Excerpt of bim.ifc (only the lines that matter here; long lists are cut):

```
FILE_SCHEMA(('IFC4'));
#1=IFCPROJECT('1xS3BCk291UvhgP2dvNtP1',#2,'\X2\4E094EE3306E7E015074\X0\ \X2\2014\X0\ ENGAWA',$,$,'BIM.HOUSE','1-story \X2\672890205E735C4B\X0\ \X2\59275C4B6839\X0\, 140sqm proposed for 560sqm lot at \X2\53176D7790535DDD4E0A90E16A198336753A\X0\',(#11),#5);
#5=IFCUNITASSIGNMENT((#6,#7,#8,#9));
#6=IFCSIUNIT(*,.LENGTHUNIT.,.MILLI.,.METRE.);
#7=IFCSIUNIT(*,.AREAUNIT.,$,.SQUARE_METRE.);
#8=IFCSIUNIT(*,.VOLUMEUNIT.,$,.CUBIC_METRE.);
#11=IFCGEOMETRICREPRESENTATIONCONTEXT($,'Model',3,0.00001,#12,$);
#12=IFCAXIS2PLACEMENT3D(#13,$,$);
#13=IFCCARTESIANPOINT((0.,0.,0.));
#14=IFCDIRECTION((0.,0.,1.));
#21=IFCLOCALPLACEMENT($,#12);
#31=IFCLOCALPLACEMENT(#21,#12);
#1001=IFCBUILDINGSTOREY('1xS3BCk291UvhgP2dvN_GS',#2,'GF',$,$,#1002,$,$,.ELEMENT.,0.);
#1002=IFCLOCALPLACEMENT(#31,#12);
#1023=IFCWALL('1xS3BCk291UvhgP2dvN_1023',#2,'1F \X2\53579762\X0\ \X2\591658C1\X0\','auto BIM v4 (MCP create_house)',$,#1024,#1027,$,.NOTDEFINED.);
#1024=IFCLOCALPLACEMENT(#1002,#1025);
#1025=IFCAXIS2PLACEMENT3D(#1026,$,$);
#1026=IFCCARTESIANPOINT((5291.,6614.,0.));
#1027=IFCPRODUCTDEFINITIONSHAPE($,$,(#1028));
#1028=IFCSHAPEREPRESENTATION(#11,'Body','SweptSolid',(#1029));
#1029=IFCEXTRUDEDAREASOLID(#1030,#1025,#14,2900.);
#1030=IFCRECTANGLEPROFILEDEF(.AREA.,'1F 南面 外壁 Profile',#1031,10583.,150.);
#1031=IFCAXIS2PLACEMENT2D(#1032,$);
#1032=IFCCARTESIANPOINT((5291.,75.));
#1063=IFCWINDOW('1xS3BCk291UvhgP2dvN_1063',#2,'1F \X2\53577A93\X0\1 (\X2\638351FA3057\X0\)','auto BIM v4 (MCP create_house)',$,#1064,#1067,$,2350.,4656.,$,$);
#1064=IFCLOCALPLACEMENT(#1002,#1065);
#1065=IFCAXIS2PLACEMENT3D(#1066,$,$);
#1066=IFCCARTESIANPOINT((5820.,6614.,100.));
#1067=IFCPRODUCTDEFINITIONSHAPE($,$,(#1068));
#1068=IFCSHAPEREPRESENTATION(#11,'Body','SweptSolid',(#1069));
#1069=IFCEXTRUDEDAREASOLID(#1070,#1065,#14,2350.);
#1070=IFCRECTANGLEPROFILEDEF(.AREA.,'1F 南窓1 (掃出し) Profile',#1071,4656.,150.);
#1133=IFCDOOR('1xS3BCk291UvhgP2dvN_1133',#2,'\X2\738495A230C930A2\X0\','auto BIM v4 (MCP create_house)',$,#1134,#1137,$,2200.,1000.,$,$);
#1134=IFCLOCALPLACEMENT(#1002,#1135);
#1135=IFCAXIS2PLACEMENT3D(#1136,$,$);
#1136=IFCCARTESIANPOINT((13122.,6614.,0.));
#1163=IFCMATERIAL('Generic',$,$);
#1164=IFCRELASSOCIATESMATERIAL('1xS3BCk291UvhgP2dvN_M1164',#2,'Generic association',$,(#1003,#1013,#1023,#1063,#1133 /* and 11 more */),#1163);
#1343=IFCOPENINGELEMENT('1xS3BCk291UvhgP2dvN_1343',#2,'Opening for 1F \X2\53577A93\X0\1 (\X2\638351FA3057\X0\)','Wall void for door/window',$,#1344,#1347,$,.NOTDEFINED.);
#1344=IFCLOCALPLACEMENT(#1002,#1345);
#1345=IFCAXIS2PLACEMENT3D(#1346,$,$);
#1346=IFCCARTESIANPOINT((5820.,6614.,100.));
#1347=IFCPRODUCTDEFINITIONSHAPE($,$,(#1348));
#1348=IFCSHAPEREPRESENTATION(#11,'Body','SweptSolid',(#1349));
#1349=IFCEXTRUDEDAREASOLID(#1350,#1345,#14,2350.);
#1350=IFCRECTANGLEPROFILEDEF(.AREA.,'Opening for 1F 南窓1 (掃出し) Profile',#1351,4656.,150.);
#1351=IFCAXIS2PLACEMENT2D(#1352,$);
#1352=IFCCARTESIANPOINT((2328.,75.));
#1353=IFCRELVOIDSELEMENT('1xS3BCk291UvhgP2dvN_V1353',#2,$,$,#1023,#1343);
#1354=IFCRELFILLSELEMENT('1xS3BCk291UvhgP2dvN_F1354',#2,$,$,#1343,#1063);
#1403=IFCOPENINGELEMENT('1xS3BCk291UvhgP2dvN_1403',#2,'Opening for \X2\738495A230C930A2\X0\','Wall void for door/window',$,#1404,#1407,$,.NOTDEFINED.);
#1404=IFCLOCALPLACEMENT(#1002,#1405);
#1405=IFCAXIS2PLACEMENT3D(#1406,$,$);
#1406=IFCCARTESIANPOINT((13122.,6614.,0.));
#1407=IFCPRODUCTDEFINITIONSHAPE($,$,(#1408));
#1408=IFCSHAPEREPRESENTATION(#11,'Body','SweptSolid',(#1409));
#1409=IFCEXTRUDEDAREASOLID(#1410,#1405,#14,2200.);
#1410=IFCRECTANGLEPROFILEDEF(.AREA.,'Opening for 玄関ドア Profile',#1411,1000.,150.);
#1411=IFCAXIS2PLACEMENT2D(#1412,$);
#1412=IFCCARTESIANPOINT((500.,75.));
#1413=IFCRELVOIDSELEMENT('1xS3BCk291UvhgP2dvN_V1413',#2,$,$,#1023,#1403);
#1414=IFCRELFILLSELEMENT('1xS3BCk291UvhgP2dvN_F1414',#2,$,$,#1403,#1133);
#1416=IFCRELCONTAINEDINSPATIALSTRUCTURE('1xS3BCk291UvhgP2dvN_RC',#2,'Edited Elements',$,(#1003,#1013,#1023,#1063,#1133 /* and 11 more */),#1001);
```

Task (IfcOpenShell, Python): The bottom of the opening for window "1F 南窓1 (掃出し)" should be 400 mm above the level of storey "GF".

```python
import numpy as np
import ifcopenshell
import ifcopenshell.api.geometry
import ifcopenshell.geom
import ifcopenshell.util.element
import ifcopenshell.util.placement
import ifcopenshell.util.shape
import ifcopenshell.util.unit

model = ifcopenshell.open("bim.ifc")
unit_scale = ifcopenshell.util.unit.calculate_unit_scale(model)

window = model.by_guid("1xS3BCk291UvhgP2dvN_1063")
opening = window.FillsVoids[0].RelatingOpeningElement
storey = ifcopenshell.util.element.get_container(window, ifc_class="IfcBuildingStorey")
level = ifcopenshell.util.placement.get_local_placement(storey.ObjectPlacement)[2, 3]

# The opening's origin need not be at the sill, so measure its lowest point.
shape = ifcopenshell.geom.create_shape(ifcopenshell.geom.settings(), opening)
bottom = ifcopenshell.util.shape.get_shape_bottom_elevation(shape, shape.geometry) / unit_scale
dz = level + 0.4 / unit_scale - bottom

shift = np.array([0.0, 0.0, dz])
# The window is not placed relative to its opening, so move both.
for product in (opening, window):
    matrix = ifcopenshell.util.placement.get_local_placement(product.ObjectPlacement)
    matrix[:3, 3] += shift
    ifcopenshell.api.geometry.edit_object_placement(model, product=product, matrix=matrix, is_si=False)

print(f"moved by {dz * unit_scale:+.3f} m")

model.write("bim_edited.ifc")
```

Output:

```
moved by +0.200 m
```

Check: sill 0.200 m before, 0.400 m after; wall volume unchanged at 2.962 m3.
